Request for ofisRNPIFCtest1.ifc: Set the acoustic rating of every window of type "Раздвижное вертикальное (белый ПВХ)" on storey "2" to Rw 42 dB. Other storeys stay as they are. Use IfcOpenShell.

First a look at what the model holds.

```python
import ifcopenshell
import ifcopenshell.util.element

model = ifcopenshell.open("ofisRNPIFCtest1.ifc")
print(model.schema)
storey = next(s for s in model.by_type("IfcBuildingStorey") if s.Name == "2")
windows = [e for e in ifcopenshell.util.element.get_decomposition(storey) if e.is_a("IfcWindow")]
seen = {}
for e in windows:
    element_type = ifcopenshell.util.element.get_type(e)
    key = (element_type.Name if element_type != e and element_type else None, ifcopenshell.util.element.get_pset(e, "Pset_WindowCommon", "AcousticRating"))
    seen[key] = seen.get(key, 0) + 1
for (name, value), count in sorted(seen.items(), key=str):
    print(count, "x", name, "|", value)
```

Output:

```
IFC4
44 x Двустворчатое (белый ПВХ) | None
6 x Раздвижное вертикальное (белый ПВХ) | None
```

```python
import ifcopenshell
import ifcopenshell.api.pset
import ifcopenshell.util.element

model = ifcopenshell.open("ofisRNPIFCtest1.ifc")

storey = next(s for s in model.by_type("IfcBuildingStorey") if s.Name == "2")
windows = [e for e in ifcopenshell.util.element.get_decomposition(storey) if e.is_a("IfcWindow")]

count = 0
for e in windows:
    element_type = ifcopenshell.util.element.get_type(e)
    if element_type in (None, e) or element_type.Name != "Раздвижное вертикальное (белый ПВХ)":
        continue
    # add_pset returns the element's existing set when there is one.
    pset = ifcopenshell.api.pset.add_pset(model, product=e, name="Pset_WindowCommon")
    ifcopenshell.api.pset.edit_pset(model, pset=pset, properties={"AcousticRating": "Rw 42 dB"})
    count += 1

print(count, "windows updated")

model.write("ofisRNPIFCtest1-out.ifc")
```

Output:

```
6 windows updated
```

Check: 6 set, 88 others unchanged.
